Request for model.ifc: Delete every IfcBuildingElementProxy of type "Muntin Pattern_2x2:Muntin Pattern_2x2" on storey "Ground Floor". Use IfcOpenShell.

First a look at what the model holds.

```python
import ifcopenshell
import ifcopenshell.util.element

model = ifcopenshell.open("model.ifc")
print(model.schema)
storey = next(s for s in model.by_type("IfcBuildingStorey") if s.Name == "Ground Floor")
proxies = [e for e in ifcopenshell.util.element.get_decomposition(storey) if e.is_a("IfcBuildingElementProxy")]
seen = {}
for e in proxies:
    element_type = ifcopenshell.util.element.get_type(e)
    name = element_type.Name if element_type not in (None, e) else None
    seen[name] = seen.get(name, 0) + 1
for name, count in sorted(seen.items(), key=str):
    print(count, "x", name)
```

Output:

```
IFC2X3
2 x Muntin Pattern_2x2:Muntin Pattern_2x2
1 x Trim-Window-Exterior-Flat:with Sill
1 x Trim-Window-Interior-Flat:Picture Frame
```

```python
import ifcopenshell
import ifcopenshell.api.root
import ifcopenshell.util.element

model = ifcopenshell.open("model.ifc")

storey = next(s for s in model.by_type("IfcBuildingStorey") if s.Name == "Ground Floor")
proxies = [e for e in ifcopenshell.util.element.get_decomposition(storey) if e.is_a("IfcBuildingElementProxy")]
targets = [e for e in proxies if (t := ifcopenshell.util.element.get_type(e)) not in (None, e) and t.Name == "Muntin Pattern_2x2:Muntin Pattern_2x2"]

for e in targets:
    ifcopenshell.api.root.remove_product(model, product=e)
print(len(targets), "removed")

model.write("model_updated.ifc")
```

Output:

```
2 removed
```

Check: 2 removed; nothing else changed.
